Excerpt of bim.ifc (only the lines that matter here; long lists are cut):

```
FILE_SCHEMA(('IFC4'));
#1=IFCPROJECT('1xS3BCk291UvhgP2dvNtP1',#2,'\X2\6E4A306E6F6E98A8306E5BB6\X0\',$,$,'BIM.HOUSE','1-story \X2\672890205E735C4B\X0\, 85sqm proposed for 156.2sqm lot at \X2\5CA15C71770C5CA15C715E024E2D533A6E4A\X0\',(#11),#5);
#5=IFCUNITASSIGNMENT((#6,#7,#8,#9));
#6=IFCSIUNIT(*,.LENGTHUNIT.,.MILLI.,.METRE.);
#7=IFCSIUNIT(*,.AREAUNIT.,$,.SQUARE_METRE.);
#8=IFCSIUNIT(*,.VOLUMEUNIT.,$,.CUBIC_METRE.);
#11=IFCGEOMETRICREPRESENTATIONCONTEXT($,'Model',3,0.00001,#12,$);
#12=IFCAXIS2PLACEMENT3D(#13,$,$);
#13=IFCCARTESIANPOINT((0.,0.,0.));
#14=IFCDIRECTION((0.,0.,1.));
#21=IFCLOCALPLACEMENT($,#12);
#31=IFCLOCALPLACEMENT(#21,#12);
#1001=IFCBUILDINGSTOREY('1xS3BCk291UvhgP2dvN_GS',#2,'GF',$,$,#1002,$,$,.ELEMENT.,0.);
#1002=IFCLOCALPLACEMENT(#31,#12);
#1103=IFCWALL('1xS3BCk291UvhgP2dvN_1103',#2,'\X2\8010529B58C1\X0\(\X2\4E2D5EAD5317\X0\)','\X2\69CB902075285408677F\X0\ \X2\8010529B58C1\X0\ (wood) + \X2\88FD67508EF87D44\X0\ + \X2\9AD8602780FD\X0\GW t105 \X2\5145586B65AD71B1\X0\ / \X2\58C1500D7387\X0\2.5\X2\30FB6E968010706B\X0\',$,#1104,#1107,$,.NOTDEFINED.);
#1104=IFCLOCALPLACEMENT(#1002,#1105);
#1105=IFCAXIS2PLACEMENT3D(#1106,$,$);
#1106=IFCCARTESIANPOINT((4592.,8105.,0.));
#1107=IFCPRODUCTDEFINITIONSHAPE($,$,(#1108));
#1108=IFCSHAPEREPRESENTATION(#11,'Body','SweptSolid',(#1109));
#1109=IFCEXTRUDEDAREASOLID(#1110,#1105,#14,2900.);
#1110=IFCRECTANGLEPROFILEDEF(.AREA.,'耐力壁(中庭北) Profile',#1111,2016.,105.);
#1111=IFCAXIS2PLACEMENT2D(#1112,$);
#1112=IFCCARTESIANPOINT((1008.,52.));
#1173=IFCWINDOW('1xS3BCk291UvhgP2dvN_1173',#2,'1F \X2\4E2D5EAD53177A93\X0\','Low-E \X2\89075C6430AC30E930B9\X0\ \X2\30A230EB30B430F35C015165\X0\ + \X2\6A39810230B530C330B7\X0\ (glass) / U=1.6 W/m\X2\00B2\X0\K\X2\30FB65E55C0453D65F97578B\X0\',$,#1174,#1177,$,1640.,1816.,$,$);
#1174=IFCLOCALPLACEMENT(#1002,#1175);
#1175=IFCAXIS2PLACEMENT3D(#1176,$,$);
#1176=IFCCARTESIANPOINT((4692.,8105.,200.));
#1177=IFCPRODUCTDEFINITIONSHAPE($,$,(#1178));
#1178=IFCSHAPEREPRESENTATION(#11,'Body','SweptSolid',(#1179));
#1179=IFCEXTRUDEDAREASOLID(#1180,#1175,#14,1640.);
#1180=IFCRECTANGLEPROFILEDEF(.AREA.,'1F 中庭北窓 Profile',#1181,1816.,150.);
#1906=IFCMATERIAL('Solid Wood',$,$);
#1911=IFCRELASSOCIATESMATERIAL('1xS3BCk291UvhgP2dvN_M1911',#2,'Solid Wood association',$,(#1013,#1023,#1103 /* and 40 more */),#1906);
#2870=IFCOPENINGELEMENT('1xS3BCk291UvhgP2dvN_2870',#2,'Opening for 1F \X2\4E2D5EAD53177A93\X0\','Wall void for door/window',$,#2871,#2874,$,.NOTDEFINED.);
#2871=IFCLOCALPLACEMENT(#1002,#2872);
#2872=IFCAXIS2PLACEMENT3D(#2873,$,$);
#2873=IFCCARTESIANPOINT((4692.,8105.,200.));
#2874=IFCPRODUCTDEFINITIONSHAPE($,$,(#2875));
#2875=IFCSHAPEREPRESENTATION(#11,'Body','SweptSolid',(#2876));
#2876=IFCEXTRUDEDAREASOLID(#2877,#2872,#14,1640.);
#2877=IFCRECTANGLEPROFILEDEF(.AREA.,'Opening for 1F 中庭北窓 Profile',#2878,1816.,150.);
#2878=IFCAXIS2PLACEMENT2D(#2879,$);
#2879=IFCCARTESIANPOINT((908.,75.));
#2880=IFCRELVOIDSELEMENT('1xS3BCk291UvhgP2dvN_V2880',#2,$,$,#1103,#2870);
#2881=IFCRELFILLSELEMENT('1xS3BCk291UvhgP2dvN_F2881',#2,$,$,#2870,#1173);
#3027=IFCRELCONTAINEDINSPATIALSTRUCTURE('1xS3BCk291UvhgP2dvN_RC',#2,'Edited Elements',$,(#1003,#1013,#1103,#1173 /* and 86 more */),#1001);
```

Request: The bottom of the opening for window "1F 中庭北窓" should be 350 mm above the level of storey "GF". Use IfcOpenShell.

```python
import numpy as np
import ifcopenshell
import ifcopenshell.api.geometry
import ifcopenshell.geom
import ifcopenshell.util.element
import ifcopenshell.util.placement
import ifcopenshell.util.shape
import ifcopenshell.util.unit

model = ifcopenshell.open("bim.ifc")
unit_scale = ifcopenshell.util.unit.calculate_unit_scale(model)

window = model.by_guid("1xS3BCk291UvhgP2dvN_1173")
opening = window.FillsVoids[0].RelatingOpeningElement
storey = ifcopenshell.util.element.get_container(window, ifc_class="IfcBuildingStorey")
level = ifcopenshell.util.placement.get_local_placement(storey.ObjectPlacement)[2, 3]

# The opening's origin need not be at the sill, so measure its lowest point.
shape = ifcopenshell.geom.create_shape(ifcopenshell.geom.settings(), opening)
bottom = ifcopenshell.util.shape.get_shape_bottom_elevation(shape, shape.geometry) / unit_scale
dz = level + 350.0 - bottom

shift = np.array([0.0, 0.0, dz])
# The window is not placed relative to its opening, so move both.
for product in (opening, window):
    matrix = ifcopenshell.util.placement.get_local_placement(product.ObjectPlacement)
    matrix[:3, 3] += shift
    ifcopenshell.api.geometry.edit_object_placement(model, product=product, matrix=matrix, is_si=False)

print(f"moved by {dz * unit_scale:+.3f} m")

model.write("bim-out.ifc")
```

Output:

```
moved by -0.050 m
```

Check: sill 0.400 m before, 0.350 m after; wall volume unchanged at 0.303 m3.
